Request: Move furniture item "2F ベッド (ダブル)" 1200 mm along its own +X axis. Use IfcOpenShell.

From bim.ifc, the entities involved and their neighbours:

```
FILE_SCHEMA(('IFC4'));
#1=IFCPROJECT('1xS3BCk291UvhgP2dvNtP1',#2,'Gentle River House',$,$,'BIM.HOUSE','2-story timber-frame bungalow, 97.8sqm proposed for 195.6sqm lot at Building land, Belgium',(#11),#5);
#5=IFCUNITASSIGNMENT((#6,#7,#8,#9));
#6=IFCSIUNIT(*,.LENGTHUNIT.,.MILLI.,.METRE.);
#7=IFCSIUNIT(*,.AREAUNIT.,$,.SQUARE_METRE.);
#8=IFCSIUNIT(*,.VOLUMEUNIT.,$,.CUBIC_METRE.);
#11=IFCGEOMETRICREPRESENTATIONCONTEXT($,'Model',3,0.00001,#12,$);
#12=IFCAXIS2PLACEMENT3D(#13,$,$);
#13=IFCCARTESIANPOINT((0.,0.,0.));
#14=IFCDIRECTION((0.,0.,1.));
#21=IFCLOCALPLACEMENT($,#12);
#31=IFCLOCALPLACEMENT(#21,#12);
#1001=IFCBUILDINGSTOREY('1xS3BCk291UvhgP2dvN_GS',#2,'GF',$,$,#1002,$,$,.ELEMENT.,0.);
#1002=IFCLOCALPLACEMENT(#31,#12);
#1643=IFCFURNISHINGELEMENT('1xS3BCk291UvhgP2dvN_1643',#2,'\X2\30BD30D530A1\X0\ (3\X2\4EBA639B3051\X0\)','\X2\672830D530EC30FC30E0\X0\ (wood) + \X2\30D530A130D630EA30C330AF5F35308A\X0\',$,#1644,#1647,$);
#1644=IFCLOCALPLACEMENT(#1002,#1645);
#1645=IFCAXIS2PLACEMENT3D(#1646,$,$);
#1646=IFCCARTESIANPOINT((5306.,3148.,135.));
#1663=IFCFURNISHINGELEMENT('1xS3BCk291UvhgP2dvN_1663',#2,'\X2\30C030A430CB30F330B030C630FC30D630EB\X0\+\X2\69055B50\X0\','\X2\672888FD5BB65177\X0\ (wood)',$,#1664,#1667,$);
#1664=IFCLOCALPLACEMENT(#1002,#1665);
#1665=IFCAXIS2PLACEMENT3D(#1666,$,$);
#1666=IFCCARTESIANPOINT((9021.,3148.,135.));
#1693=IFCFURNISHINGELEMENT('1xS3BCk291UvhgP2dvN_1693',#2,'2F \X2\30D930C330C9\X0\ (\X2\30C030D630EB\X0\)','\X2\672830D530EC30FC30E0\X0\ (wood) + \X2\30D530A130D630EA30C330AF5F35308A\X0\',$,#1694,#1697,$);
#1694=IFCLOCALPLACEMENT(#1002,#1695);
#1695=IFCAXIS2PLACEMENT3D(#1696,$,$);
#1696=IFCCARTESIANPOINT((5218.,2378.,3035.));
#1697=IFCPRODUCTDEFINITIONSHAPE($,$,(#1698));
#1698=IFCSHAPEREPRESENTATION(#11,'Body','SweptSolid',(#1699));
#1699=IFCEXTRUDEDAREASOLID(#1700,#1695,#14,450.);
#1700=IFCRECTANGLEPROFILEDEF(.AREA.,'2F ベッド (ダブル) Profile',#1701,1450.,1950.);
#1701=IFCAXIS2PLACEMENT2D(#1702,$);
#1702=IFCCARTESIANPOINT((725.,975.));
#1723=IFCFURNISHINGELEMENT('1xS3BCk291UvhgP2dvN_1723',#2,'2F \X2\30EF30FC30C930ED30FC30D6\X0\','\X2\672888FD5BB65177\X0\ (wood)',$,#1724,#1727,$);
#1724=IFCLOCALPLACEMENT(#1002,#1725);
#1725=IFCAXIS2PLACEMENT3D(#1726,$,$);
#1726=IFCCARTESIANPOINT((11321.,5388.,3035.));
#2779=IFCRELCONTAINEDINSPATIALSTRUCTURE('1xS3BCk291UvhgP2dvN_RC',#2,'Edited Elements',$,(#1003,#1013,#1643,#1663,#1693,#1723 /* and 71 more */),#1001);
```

```python
import ifcopenshell
import ifcopenshell.api.geometry
import ifcopenshell.util.placement
import ifcopenshell.util.unit

model = ifcopenshell.open("bim.ifc")
unit_scale = ifcopenshell.util.unit.calculate_unit_scale(model)

item = model.by_guid("1xS3BCk291UvhgP2dvN_1693")
matrix = ifcopenshell.util.placement.get_local_placement(item.ObjectPlacement)
matrix[:3, 3] += matrix[:3, 0] * 1.2 / unit_scale
ifcopenshell.api.geometry.edit_object_placement(model, product=item, matrix=matrix, is_si=False)

print(ifcopenshell.util.placement.get_local_placement(item.ObjectPlacement).round(3) + 0.0)

model.write("bim_v2.ifc")
```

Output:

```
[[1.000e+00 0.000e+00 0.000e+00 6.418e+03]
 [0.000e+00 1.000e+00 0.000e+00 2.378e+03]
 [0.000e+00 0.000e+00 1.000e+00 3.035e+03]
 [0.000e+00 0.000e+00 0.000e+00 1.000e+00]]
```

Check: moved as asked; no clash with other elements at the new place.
